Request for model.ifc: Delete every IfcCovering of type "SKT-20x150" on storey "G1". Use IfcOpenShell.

First a look at what the model holds.

```python
import ifcopenshell
import ifcopenshell.util.element

model = ifcopenshell.open("model.ifc")
print(model.schema)
storey = next(s for s in model.by_type("IfcBuildingStorey") if s.Name == "G1")
coverings = [e for e in ifcopenshell.util.element.get_decomposition(storey) if e.is_a("IfcCovering")]
seen = {}
for e in coverings:
    element_type = ifcopenshell.util.element.get_type(e)
    name = element_type.Name if element_type not in (None, e) else None
    seen[name] = seen.get(name, 0) + 1
for name, count in sorted(seen.items(), key=str):
    print(count, "x", name)
```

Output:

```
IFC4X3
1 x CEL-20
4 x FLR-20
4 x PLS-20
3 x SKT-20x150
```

```python
import ifcopenshell
import ifcopenshell.api.root
import ifcopenshell.util.element

model = ifcopenshell.open("model.ifc")

storey = next(s for s in model.by_type("IfcBuildingStorey") if s.Name == "G1")
coverings = [e for e in ifcopenshell.util.element.get_decomposition(storey) if e.is_a("IfcCovering")]
targets = [e for e in coverings if (t := ifcopenshell.util.element.get_type(e)) not in (None, e) and t.Name == "SKT-20x150"]

for e in targets:
    ifcopenshell.api.root.remove_product(model, product=e)
print(len(targets), "removed")

model.write("model_rev.ifc")
```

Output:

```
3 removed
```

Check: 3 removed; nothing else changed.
